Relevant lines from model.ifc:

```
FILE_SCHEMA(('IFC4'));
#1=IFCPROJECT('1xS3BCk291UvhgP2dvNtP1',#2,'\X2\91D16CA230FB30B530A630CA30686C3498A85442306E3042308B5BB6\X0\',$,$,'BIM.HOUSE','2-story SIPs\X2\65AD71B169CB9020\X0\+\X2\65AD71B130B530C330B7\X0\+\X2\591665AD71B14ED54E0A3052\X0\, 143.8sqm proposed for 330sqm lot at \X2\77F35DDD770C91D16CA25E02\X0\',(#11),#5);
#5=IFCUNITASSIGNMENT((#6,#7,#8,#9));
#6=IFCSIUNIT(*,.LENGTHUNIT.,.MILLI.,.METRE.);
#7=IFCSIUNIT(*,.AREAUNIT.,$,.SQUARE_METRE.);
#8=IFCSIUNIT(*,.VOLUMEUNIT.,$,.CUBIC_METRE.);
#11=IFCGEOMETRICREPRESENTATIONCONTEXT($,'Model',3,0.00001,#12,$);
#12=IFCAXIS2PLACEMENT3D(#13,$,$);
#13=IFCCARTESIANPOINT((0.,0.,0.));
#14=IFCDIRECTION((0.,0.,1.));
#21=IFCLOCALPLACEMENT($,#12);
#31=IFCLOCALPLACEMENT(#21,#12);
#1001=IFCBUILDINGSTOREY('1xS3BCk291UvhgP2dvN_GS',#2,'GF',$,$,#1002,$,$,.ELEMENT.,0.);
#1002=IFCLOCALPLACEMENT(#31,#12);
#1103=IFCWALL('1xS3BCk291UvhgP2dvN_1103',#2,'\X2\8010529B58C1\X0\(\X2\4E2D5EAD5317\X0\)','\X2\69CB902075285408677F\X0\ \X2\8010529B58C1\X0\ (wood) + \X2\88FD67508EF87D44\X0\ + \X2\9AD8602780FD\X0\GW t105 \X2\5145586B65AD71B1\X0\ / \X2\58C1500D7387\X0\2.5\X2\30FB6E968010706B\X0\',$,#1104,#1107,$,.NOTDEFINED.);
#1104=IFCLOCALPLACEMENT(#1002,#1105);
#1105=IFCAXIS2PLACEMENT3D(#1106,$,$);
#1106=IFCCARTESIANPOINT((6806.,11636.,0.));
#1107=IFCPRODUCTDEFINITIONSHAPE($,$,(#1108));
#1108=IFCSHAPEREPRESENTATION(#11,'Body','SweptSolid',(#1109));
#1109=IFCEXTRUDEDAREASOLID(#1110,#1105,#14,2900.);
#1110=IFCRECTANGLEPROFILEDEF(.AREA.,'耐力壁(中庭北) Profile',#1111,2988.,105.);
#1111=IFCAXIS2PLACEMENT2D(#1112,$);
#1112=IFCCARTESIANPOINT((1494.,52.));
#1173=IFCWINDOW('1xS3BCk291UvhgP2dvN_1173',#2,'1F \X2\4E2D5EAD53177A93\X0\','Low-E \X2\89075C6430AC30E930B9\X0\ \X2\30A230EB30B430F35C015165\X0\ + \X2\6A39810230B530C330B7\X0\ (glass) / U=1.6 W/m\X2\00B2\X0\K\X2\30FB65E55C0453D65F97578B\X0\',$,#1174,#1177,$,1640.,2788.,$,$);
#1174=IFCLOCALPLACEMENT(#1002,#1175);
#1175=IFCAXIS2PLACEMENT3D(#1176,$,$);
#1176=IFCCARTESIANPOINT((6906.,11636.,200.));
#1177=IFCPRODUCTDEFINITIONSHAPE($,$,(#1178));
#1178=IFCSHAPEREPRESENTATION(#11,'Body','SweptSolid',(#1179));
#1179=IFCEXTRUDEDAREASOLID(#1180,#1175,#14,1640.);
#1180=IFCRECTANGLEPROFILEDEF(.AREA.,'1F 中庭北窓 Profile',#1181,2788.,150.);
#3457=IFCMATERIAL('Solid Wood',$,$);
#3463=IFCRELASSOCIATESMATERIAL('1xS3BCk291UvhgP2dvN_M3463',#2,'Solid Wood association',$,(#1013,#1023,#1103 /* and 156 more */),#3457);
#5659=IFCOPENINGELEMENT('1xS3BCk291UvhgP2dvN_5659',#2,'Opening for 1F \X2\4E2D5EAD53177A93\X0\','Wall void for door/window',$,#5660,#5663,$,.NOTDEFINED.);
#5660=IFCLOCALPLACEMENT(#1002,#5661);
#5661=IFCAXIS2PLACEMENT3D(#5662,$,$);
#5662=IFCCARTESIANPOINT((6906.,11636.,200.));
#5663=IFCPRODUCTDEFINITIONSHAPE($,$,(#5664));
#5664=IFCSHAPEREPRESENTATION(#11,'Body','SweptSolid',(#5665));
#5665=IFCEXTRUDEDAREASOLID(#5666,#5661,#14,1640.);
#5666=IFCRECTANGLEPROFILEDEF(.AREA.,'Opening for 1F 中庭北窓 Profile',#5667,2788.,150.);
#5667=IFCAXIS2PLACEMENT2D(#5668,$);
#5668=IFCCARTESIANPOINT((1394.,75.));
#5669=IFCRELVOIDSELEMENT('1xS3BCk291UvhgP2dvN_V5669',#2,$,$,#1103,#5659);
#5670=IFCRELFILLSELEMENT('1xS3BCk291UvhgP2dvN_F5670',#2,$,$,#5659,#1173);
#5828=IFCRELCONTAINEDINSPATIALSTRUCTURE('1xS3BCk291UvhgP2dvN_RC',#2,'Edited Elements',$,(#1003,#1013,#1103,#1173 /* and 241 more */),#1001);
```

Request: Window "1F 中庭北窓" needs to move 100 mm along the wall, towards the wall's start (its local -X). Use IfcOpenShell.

```python
import ifcopenshell
import ifcopenshell.api.geometry
import ifcopenshell.util.placement
import ifcopenshell.util.unit

model = ifcopenshell.open("model.ifc")
unit_scale = ifcopenshell.util.unit.calculate_unit_scale(model)

window = model.by_guid("1xS3BCk291UvhgP2dvN_1173")
opening = window.FillsVoids[0].RelatingOpeningElement
wall = opening.VoidsElements[0].RelatingBuildingElement

wall_matrix = ifcopenshell.util.placement.get_local_placement(wall.ObjectPlacement)
shift = wall_matrix[:3, 0] * -0.1 / unit_scale
before = ifcopenshell.util.placement.get_local_placement(window.ObjectPlacement)[:3, 3].copy()

# The window is not placed relative to its opening, so move both.
for product in (opening, window):
    matrix = ifcopenshell.util.placement.get_local_placement(product.ObjectPlacement)
    matrix[:3, 3] += shift
    ifcopenshell.api.geometry.edit_object_placement(model, product=product, matrix=matrix, is_si=False)

after = ifcopenshell.util.placement.get_local_placement(window.ObjectPlacement)[:3, 3]
print("window moved by", (after - before).round(3) + 0.0)

model.write("model_edited.ifc")
```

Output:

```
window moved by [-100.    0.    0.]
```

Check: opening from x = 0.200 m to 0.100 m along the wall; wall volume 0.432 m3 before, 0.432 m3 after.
